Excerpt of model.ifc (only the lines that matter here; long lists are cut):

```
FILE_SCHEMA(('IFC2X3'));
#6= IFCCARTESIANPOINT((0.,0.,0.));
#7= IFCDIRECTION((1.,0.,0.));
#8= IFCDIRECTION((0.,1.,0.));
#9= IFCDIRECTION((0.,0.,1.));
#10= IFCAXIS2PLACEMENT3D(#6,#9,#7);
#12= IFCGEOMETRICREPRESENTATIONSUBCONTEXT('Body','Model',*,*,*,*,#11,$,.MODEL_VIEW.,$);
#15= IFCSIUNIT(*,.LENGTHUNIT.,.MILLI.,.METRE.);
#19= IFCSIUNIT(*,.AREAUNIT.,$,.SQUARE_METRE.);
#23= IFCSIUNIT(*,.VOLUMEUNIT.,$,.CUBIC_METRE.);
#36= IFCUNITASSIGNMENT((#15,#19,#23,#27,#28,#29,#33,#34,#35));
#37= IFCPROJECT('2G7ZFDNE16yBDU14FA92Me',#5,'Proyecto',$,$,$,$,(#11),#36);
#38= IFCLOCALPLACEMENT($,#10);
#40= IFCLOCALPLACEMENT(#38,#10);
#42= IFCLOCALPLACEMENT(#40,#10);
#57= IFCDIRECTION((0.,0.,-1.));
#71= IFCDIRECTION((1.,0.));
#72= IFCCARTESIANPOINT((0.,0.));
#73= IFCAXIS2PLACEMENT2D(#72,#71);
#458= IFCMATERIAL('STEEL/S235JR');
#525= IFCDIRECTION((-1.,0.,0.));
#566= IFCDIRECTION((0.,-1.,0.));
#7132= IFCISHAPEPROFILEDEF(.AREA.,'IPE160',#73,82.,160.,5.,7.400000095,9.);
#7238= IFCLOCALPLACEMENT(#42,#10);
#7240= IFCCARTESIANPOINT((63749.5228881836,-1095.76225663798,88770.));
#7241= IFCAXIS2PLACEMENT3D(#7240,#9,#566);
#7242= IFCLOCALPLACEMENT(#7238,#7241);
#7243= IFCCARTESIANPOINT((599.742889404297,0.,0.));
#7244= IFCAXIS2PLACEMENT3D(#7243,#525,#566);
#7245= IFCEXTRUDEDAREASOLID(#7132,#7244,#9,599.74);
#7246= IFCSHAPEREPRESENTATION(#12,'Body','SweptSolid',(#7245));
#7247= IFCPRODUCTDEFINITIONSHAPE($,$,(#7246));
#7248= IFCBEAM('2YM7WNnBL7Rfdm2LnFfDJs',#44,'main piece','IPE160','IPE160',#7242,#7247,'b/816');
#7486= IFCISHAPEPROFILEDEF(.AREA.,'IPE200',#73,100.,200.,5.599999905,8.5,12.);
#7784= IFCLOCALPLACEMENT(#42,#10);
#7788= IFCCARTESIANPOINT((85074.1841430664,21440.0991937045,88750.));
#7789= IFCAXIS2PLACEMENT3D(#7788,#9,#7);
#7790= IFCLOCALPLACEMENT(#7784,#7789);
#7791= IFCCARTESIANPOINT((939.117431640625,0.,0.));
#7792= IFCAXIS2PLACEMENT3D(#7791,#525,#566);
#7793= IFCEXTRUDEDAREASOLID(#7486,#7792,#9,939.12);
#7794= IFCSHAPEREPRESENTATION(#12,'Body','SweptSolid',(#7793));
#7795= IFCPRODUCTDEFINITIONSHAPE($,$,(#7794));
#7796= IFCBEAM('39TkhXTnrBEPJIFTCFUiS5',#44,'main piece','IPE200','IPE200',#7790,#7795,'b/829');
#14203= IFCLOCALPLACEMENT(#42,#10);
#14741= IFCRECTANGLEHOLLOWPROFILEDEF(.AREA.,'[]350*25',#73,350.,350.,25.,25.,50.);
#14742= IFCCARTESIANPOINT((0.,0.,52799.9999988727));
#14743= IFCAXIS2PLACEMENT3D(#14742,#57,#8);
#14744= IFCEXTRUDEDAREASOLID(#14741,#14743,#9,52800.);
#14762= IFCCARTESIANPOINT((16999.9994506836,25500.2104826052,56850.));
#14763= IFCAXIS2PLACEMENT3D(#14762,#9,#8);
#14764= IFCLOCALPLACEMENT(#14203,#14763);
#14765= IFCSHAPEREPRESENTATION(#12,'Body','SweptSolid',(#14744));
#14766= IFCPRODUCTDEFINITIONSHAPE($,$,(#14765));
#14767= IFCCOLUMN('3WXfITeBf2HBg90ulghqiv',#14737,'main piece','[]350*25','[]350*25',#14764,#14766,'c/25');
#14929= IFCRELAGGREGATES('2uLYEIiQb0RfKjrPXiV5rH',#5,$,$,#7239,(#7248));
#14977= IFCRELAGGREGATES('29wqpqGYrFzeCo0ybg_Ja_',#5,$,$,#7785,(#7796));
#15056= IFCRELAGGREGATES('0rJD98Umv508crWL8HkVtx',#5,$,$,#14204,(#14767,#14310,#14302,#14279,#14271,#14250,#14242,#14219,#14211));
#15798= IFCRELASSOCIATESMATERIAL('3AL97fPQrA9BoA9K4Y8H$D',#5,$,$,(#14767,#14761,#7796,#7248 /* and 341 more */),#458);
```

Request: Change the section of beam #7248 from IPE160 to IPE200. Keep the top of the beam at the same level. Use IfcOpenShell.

```python
import ifcopenshell
import ifcopenshell.util.element
import ifcopenshell.util.representation

model = ifcopenshell.open("model.ifc")

member = model.by_guid("2YM7WNnBL7Rfdm2LnFfDJs")
source = next(p for p in model.by_type("IfcIShapeProfileDef") if p.ProfileName == "IPE200")

body = ifcopenshell.util.representation.get_representation(member, "Model", "Body")
solid = body.Items[0]
old_profile = solid.SweptArea

# Copy the section's sizes but keep this member's own profile position.
profile = ifcopenshell.util.element.copy(model, source)
# Profiles are centred, so shift by half the change in depth to hold the top.
shift = (old_profile.OverallDepth - profile.OverallDepth) / 2
x, y = old_profile.Position.Location.Coordinates
up = (0.0, 1.0)  # upwards, in the solid's own plane
location = model.createIfcCartesianPoint((x + up[0] * shift, y + up[1] * shift))
profile.Position = model.createIfcAxis2Placement2D(location, old_profile.Position.RefDirection)
solid.SweptArea = profile
if not model.get_total_inverses(old_profile):
    ifcopenshell.util.element.remove_deep2(model, old_profile)
member.Description = member.Description.replace("IPE160", "IPE200")
member.ObjectType = member.ObjectType.replace("IPE160", "IPE200")

print(solid.SweptArea)

model.write("model_edited.ifc")
```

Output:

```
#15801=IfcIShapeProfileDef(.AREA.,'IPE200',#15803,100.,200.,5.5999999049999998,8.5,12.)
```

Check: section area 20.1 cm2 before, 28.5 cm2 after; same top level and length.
